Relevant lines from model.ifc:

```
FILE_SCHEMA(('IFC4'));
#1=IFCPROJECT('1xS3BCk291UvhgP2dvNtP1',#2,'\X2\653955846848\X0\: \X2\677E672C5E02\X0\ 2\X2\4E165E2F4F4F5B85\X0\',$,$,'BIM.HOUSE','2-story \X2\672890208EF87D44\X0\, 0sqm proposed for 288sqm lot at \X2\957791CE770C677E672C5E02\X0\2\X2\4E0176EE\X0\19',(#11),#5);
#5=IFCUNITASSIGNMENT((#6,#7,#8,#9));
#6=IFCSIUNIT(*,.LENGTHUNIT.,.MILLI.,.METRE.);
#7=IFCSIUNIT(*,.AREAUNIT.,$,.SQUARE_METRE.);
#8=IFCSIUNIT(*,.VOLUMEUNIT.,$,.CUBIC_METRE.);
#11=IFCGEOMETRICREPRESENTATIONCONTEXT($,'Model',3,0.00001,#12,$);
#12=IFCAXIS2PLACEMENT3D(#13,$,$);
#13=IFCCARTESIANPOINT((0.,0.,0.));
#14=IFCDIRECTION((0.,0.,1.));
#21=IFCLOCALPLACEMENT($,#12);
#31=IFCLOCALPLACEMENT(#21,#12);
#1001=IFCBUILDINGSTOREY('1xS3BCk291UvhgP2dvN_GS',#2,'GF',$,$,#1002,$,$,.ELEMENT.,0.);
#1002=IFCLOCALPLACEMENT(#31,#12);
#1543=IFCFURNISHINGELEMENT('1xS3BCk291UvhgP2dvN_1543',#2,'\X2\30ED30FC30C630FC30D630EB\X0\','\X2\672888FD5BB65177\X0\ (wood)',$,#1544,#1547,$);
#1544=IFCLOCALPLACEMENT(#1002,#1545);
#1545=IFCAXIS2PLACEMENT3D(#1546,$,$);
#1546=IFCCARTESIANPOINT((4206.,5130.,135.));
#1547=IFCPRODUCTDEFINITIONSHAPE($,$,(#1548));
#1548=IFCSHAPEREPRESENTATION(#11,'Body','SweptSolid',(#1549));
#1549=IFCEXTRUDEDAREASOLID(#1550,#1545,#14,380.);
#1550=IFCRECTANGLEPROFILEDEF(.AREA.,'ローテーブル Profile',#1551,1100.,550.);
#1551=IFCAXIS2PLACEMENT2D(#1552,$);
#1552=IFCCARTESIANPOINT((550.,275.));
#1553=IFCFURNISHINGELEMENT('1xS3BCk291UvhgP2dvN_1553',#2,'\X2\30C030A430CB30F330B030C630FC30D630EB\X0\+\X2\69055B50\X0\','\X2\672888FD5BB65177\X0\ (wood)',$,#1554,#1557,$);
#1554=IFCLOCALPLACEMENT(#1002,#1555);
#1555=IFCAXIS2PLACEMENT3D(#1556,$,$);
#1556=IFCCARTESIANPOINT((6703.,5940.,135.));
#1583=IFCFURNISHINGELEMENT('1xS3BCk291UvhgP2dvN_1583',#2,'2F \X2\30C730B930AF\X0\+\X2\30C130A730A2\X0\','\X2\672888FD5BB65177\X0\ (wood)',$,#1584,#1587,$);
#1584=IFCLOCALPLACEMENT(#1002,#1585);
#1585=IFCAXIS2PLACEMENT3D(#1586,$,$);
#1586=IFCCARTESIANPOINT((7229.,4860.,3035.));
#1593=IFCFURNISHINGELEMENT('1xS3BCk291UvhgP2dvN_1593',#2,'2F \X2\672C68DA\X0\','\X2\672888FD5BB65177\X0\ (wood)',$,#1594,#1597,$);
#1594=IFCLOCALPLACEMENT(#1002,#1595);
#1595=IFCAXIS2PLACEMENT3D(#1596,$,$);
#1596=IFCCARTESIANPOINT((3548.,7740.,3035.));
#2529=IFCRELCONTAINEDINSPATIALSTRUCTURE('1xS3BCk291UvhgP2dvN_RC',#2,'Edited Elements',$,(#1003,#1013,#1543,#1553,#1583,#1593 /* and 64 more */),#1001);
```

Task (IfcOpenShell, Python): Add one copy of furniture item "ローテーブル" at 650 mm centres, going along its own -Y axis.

```python
import ifcopenshell
import ifcopenshell.api.geometry
import ifcopenshell.api.root
import ifcopenshell.util.element
import ifcopenshell.util.placement

model = ifcopenshell.open("model.ifc")


def reuse_history(source, copy):
    """copy_class also copies each property set's owner history, people and application; keep the originals."""
    for rel in copy.IsDefinedBy:
        if rel.is_a("IfcRelDefinesByProperties") and (history := rel.RelatingPropertyDefinition.OwnerHistory):
            rel.RelatingPropertyDefinition.OwnerHistory = source.OwnerHistory
            ifcopenshell.util.element.remove_deep2(model, history)


source = model.by_guid("1xS3BCk291UvhgP2dvN_1543")
base = ifcopenshell.util.placement.get_local_placement(source.ObjectPlacement)
step = -base[:3, 1] * 650.0

for i in range(1, 2):
    copy = ifcopenshell.api.root.copy_class(model, product=source)
    copy.Representation = ifcopenshell.util.element.copy_deep(
        model, source.Representation, exclude=["IfcGeometricRepresentationContext", "IfcRepresentationMap"]
    )
    reuse_history(source, copy)
    matrix = base.copy()
    matrix[:3, 3] += i * step
    print("added at", matrix[:3, 3].round(3) + 0.0)
    ifcopenshell.api.geometry.edit_object_placement(model, product=copy, matrix=matrix, is_si=False)

model.write("model_edited.ifc")
```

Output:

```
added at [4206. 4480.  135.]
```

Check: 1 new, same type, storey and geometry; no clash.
